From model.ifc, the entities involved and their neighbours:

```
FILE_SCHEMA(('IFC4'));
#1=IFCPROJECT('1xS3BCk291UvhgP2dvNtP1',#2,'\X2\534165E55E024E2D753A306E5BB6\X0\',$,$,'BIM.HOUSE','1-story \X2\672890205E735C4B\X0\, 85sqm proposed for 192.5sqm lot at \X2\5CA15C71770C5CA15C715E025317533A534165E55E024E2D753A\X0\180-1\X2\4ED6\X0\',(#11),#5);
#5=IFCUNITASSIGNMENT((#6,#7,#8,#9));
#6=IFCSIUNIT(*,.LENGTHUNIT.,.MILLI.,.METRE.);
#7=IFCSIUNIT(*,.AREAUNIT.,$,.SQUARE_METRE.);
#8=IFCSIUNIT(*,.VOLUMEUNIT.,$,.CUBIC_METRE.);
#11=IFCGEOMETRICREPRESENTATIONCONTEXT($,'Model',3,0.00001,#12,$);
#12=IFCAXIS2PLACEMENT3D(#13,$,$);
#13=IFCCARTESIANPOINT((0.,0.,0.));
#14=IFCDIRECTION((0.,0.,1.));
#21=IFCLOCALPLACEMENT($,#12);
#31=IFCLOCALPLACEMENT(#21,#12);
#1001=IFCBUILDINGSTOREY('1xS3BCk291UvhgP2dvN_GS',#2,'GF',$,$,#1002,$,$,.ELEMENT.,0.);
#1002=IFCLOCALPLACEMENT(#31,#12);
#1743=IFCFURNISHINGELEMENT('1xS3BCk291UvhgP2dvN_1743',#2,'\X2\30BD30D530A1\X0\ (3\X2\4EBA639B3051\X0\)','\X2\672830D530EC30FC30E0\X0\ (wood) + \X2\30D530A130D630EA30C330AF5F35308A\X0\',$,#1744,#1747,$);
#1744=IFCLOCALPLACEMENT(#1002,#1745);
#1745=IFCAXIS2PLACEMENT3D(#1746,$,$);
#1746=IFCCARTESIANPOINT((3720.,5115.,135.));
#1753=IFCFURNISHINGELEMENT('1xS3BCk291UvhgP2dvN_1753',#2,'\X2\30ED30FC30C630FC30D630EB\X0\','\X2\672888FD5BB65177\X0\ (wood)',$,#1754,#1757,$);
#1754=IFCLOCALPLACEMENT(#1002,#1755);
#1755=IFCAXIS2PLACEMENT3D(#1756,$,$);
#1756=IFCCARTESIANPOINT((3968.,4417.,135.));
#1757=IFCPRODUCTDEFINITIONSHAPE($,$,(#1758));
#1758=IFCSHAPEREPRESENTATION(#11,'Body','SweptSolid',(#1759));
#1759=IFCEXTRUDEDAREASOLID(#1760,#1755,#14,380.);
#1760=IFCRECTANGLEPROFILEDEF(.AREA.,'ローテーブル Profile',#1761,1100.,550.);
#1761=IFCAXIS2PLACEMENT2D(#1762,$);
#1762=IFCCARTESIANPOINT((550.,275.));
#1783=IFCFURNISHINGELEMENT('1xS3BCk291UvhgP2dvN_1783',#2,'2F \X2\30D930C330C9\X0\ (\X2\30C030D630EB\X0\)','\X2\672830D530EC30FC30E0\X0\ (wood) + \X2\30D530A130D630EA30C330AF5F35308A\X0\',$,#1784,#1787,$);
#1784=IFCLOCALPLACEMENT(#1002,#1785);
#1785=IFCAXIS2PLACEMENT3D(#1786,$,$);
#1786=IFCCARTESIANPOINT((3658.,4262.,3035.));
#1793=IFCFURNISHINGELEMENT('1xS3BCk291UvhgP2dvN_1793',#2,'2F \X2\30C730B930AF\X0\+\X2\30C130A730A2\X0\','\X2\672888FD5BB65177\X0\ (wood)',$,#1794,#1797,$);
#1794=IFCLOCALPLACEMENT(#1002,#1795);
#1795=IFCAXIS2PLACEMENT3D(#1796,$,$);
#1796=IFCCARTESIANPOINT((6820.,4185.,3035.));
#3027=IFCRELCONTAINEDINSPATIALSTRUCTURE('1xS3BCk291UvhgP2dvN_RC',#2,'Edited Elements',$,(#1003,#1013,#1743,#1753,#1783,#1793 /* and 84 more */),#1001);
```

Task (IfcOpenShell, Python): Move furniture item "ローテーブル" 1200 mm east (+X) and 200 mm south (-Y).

```python
import ifcopenshell
import ifcopenshell.api.geometry
import ifcopenshell.util.placement

model = ifcopenshell.open("model.ifc")

item = model.by_guid("1xS3BCk291UvhgP2dvN_1753")
matrix = ifcopenshell.util.placement.get_local_placement(item.ObjectPlacement)
matrix[0, 3] += 1200.0
matrix[1, 3] -= 200.0
ifcopenshell.api.geometry.edit_object_placement(model, product=item, matrix=matrix, is_si=False)

print(ifcopenshell.util.placement.get_local_placement(item.ObjectPlacement).round(3) + 0.0)

model.write("model_edited.ifc")
```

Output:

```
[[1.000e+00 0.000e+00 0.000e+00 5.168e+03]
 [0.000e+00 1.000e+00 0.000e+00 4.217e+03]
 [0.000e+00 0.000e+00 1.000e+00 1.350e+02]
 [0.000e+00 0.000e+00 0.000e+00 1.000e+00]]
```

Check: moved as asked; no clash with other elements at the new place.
